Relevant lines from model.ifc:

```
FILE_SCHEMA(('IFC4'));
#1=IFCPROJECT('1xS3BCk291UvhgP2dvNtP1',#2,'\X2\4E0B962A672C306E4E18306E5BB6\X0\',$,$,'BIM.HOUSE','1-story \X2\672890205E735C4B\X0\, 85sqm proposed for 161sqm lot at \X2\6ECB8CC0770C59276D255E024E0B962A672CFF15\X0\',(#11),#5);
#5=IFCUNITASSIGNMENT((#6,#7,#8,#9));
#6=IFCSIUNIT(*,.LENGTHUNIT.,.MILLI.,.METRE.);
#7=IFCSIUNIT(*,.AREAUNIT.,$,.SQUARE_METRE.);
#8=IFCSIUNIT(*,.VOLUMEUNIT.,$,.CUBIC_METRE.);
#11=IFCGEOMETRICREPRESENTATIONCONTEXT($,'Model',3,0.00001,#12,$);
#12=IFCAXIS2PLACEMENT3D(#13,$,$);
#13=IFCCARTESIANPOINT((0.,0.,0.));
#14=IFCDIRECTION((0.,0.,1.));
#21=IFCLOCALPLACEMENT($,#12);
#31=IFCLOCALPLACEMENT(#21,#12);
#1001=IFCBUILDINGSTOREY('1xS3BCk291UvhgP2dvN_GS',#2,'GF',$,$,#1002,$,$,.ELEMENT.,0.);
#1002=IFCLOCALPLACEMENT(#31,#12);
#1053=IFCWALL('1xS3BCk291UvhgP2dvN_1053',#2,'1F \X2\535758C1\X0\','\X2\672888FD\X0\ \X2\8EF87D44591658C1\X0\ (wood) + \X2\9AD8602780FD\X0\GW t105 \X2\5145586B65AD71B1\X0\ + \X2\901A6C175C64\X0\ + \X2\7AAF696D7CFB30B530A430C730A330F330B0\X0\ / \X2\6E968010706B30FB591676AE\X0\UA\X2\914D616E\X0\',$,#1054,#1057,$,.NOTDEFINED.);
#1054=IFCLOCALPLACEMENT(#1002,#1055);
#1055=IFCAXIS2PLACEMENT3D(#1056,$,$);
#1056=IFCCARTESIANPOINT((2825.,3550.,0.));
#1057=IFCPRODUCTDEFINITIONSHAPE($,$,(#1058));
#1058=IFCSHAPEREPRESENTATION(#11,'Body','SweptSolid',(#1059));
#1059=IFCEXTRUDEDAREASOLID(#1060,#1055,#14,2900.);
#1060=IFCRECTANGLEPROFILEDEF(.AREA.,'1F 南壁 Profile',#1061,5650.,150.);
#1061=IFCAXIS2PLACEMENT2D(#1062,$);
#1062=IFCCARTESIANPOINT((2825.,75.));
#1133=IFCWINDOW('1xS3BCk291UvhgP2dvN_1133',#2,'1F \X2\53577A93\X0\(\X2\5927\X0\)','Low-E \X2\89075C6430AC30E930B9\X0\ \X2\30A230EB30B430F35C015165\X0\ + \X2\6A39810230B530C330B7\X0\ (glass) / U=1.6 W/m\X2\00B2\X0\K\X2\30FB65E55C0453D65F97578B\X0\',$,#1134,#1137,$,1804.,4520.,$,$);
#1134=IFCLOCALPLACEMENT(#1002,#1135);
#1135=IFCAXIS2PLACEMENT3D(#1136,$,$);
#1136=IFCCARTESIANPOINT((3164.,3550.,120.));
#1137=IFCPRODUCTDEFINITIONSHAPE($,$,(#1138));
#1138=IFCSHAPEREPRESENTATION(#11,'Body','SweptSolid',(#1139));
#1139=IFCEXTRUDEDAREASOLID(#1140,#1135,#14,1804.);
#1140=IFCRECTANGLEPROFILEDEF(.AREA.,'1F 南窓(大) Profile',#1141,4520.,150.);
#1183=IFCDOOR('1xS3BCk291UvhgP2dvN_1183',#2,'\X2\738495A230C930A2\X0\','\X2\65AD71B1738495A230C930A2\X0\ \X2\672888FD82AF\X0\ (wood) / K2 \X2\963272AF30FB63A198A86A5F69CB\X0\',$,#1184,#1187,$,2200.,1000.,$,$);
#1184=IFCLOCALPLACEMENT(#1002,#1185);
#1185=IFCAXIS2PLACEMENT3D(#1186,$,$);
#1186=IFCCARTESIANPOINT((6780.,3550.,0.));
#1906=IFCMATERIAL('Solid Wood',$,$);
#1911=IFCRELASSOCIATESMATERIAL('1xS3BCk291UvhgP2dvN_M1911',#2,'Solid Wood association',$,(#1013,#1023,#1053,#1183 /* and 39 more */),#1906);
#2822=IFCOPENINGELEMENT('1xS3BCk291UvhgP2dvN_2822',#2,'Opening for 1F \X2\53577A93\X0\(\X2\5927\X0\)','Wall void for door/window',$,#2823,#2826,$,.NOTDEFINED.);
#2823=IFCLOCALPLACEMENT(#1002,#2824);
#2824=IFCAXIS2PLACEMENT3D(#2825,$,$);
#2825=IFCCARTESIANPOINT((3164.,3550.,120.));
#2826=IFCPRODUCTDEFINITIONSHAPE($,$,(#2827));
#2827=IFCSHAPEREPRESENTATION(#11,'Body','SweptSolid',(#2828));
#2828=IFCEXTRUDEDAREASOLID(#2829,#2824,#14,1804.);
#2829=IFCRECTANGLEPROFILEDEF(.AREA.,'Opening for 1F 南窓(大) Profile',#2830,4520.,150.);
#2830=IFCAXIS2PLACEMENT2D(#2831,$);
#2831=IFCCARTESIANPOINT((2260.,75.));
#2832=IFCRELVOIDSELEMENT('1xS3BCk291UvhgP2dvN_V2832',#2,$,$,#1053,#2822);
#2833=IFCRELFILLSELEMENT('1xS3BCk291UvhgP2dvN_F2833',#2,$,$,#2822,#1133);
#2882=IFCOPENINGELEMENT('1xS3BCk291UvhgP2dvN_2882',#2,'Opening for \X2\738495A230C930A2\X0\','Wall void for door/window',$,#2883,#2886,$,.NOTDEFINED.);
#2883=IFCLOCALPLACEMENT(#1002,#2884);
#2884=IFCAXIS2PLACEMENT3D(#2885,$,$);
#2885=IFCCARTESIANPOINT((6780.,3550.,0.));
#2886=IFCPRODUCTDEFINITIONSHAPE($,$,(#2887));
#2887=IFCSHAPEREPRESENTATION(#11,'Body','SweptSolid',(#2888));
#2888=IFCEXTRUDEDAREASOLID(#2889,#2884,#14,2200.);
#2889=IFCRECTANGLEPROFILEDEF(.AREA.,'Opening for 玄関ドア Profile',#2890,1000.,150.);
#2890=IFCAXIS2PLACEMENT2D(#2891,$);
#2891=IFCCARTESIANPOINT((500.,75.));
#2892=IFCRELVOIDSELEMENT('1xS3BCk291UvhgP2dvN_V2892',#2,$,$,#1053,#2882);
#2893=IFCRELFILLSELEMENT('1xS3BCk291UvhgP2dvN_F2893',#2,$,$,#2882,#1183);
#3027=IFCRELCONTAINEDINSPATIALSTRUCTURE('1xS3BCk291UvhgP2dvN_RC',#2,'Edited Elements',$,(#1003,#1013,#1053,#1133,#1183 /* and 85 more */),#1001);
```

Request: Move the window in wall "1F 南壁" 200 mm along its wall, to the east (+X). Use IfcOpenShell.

```python
import ifcopenshell
import ifcopenshell.api.geometry
import ifcopenshell.util.placement
import ifcopenshell.util.unit

model = ifcopenshell.open("model.ifc")
unit_scale = ifcopenshell.util.unit.calculate_unit_scale(model)

window = model.by_guid("1xS3BCk291UvhgP2dvN_1133")
opening = window.FillsVoids[0].RelatingOpeningElement
wall = opening.VoidsElements[0].RelatingBuildingElement

wall_matrix = ifcopenshell.util.placement.get_local_placement(wall.ObjectPlacement)
shift = wall_matrix[:3, 0] * 0.2 / unit_scale
before = ifcopenshell.util.placement.get_local_placement(window.ObjectPlacement)[:3, 3].copy()

# The window is not placed relative to its opening, so move both.
for product in (opening, window):
    matrix = ifcopenshell.util.placement.get_local_placement(product.ObjectPlacement)
    matrix[:3, 3] += shift
    ifcopenshell.api.geometry.edit_object_placement(model, product=product, matrix=matrix, is_si=False)

after = ifcopenshell.util.placement.get_local_placement(window.ObjectPlacement)[:3, 3]
print("window moved by", (after - before).round(3) + 0.0)

model.write("model_edited.ifc")
```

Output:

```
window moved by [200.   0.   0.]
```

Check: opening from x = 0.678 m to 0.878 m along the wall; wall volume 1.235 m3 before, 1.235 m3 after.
